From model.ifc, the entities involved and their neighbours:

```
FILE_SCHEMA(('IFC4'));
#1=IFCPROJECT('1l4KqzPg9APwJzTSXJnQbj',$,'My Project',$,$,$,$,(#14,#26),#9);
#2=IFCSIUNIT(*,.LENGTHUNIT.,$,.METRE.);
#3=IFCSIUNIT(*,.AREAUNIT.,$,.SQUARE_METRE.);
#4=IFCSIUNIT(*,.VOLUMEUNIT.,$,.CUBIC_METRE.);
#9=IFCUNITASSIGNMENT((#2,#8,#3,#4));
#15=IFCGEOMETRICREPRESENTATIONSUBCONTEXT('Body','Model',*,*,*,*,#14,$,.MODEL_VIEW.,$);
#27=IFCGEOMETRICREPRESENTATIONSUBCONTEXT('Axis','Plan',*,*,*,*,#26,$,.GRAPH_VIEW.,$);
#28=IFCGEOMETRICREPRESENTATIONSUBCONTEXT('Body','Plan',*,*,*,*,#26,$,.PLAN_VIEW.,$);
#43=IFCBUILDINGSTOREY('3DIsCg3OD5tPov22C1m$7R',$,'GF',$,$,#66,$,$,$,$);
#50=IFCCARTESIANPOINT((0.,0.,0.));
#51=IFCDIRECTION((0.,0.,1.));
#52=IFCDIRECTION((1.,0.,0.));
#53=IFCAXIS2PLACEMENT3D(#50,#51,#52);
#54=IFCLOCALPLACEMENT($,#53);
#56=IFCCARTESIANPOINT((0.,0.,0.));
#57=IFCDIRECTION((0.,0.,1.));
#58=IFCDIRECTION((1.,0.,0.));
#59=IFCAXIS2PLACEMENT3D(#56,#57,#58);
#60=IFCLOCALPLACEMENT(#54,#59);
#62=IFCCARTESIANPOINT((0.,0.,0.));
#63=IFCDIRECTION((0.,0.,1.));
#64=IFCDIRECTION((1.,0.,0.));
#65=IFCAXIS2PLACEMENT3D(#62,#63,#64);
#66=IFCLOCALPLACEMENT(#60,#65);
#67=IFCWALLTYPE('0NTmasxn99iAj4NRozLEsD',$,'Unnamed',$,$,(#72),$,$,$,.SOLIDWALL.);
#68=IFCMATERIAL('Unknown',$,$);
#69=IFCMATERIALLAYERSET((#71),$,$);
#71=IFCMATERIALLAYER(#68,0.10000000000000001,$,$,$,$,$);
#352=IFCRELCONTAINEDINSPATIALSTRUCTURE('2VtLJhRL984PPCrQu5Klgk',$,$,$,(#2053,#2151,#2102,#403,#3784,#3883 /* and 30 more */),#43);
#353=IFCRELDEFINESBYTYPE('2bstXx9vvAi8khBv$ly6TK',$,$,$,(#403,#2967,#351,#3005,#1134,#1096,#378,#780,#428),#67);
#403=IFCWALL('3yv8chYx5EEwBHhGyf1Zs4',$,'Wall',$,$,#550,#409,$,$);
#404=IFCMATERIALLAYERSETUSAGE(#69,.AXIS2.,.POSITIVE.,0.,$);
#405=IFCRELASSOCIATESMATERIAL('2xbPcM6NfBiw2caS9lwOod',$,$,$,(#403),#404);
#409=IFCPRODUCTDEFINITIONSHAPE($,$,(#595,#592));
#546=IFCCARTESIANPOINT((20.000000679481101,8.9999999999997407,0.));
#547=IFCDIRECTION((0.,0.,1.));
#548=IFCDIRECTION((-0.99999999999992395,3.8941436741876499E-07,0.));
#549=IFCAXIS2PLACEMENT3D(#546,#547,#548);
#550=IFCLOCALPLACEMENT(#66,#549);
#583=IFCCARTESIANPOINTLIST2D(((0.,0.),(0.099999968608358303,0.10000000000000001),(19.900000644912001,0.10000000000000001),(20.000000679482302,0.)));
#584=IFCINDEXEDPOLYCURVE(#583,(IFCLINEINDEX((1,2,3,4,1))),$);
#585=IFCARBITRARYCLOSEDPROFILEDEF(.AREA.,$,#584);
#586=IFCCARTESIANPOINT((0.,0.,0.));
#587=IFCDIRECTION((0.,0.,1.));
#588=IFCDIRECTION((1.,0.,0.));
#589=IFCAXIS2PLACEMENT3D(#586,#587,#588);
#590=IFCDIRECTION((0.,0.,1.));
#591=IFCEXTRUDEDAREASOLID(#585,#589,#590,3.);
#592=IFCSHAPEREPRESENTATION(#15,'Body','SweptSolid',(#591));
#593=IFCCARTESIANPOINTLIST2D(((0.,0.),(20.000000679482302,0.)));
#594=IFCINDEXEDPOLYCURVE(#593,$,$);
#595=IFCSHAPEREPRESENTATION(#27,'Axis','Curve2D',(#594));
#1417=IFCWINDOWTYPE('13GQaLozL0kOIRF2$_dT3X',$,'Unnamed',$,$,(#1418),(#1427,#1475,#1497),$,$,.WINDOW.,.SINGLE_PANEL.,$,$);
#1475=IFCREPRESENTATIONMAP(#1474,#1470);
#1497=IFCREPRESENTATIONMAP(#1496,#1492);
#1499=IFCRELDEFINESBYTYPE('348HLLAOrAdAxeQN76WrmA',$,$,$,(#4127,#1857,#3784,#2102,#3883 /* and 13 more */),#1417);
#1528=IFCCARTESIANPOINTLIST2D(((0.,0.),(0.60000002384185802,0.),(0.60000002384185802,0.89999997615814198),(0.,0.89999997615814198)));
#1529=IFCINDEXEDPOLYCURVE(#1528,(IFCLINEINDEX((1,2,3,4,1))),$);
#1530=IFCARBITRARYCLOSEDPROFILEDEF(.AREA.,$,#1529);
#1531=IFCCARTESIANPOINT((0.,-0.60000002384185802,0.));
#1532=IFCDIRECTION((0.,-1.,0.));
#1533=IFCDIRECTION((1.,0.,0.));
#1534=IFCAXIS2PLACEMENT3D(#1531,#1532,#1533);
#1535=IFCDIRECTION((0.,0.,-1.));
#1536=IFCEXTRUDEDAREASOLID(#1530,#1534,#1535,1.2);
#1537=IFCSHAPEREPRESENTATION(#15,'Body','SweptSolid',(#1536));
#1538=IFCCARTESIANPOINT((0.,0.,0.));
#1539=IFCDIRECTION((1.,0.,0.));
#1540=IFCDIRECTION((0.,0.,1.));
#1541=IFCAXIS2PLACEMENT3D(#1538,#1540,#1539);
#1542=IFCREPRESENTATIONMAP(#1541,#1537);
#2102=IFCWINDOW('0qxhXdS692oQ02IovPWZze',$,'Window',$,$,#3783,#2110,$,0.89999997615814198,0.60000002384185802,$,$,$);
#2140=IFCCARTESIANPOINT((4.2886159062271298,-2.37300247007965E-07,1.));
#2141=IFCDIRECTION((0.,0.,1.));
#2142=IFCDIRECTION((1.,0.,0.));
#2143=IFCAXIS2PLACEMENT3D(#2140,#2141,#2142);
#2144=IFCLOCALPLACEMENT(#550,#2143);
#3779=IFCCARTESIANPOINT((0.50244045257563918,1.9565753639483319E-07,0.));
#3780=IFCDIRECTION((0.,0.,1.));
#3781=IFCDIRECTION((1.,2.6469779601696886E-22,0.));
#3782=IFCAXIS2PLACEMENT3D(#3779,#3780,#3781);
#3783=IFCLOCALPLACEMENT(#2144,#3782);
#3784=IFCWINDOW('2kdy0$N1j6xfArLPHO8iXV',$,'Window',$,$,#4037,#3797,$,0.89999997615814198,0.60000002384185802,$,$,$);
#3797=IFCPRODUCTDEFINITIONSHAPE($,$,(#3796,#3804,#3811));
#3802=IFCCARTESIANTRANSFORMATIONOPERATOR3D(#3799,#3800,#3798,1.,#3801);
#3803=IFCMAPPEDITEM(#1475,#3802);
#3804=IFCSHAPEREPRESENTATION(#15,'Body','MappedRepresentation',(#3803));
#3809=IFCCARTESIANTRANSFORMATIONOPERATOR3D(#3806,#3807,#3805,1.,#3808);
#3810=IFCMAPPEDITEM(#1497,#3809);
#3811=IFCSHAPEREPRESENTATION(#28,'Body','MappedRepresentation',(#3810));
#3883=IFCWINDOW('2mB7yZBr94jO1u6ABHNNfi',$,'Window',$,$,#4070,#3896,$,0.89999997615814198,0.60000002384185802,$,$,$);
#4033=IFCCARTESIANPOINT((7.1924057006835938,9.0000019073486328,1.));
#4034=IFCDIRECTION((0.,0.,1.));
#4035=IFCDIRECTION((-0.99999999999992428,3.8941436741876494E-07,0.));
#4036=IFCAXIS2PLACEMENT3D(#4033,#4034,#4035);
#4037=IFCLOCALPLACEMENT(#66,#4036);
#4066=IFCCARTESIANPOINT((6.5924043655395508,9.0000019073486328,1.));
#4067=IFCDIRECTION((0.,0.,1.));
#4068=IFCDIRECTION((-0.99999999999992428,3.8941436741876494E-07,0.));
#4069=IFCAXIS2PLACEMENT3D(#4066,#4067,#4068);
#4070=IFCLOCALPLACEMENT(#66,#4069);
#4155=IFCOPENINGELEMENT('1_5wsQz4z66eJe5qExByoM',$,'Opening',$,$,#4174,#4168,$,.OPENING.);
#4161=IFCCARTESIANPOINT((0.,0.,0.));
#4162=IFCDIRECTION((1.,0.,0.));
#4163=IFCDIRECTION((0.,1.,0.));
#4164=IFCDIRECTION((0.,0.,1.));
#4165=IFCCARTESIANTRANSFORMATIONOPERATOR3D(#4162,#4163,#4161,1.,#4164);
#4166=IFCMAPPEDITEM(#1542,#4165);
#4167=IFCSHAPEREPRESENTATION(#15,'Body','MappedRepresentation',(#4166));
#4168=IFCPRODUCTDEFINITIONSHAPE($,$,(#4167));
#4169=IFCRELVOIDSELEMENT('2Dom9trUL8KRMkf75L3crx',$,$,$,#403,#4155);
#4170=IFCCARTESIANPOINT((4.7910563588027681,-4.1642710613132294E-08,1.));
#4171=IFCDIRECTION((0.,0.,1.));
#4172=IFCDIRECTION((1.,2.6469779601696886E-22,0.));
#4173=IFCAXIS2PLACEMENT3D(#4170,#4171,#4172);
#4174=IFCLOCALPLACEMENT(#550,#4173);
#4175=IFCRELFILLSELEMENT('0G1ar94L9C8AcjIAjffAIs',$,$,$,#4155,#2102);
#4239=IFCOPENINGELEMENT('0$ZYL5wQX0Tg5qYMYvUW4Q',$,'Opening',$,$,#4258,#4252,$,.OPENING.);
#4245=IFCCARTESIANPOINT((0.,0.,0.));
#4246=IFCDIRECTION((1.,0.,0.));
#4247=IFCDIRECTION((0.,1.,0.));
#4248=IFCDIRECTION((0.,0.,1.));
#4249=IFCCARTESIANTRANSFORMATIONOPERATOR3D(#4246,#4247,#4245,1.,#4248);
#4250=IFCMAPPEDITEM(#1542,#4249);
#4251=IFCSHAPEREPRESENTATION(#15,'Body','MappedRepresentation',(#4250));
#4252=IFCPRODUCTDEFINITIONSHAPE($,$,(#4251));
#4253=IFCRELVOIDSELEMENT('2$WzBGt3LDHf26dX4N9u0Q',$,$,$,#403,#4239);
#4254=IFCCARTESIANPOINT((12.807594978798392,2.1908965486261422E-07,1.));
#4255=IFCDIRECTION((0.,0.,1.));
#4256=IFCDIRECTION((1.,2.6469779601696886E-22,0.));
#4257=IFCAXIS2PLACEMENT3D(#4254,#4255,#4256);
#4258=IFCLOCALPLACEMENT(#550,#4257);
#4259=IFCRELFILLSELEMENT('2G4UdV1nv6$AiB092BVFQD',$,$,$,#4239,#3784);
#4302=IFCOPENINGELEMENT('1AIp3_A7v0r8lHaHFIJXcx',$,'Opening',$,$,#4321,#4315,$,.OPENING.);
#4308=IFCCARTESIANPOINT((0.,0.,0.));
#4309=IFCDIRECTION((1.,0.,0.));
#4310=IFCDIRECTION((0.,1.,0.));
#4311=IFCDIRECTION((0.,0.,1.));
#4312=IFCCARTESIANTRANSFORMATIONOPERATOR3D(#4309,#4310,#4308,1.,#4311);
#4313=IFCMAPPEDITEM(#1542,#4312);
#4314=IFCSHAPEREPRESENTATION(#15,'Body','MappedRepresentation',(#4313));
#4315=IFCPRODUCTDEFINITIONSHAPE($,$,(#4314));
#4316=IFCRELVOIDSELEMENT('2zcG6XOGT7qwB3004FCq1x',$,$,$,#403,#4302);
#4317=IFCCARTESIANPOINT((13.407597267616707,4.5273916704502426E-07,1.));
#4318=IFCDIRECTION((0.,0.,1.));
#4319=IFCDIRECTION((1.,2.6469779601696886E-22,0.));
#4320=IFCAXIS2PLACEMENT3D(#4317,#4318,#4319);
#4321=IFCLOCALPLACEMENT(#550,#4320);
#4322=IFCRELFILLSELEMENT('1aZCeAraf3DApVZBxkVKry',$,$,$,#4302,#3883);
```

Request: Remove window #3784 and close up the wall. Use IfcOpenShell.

```python
import ifcopenshell
import ifcopenshell.api.feature
import ifcopenshell.api.root
import ifcopenshell.geom
import ifcopenshell.util.shape

model = ifcopenshell.open("model.ifc")
settings = ifcopenshell.geom.settings()


def volume(element):
    """Net volume in cubic metres, openings subtracted."""
    shape = ifcopenshell.geom.create_shape(settings, element)
    return ifcopenshell.util.shape.get_volume(shape.geometry)


window = model.by_guid("2kdy0$N1j6xfArLPHO8iXV")
opening = window.FillsVoids[0].RelatingOpeningElement
wall = opening.VoidsElements[0].RelatingBuildingElement
before = volume(wall)

ifcopenshell.api.root.remove_product(model, product=window)
ifcopenshell.api.feature.remove_feature(model, feature=opening)

after = volume(wall)

print(f"wall volume {before:.3f} -> {after:.3f} m3")

model.write("model-out.ifc")
```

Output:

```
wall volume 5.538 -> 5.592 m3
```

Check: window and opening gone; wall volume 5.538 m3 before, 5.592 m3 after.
